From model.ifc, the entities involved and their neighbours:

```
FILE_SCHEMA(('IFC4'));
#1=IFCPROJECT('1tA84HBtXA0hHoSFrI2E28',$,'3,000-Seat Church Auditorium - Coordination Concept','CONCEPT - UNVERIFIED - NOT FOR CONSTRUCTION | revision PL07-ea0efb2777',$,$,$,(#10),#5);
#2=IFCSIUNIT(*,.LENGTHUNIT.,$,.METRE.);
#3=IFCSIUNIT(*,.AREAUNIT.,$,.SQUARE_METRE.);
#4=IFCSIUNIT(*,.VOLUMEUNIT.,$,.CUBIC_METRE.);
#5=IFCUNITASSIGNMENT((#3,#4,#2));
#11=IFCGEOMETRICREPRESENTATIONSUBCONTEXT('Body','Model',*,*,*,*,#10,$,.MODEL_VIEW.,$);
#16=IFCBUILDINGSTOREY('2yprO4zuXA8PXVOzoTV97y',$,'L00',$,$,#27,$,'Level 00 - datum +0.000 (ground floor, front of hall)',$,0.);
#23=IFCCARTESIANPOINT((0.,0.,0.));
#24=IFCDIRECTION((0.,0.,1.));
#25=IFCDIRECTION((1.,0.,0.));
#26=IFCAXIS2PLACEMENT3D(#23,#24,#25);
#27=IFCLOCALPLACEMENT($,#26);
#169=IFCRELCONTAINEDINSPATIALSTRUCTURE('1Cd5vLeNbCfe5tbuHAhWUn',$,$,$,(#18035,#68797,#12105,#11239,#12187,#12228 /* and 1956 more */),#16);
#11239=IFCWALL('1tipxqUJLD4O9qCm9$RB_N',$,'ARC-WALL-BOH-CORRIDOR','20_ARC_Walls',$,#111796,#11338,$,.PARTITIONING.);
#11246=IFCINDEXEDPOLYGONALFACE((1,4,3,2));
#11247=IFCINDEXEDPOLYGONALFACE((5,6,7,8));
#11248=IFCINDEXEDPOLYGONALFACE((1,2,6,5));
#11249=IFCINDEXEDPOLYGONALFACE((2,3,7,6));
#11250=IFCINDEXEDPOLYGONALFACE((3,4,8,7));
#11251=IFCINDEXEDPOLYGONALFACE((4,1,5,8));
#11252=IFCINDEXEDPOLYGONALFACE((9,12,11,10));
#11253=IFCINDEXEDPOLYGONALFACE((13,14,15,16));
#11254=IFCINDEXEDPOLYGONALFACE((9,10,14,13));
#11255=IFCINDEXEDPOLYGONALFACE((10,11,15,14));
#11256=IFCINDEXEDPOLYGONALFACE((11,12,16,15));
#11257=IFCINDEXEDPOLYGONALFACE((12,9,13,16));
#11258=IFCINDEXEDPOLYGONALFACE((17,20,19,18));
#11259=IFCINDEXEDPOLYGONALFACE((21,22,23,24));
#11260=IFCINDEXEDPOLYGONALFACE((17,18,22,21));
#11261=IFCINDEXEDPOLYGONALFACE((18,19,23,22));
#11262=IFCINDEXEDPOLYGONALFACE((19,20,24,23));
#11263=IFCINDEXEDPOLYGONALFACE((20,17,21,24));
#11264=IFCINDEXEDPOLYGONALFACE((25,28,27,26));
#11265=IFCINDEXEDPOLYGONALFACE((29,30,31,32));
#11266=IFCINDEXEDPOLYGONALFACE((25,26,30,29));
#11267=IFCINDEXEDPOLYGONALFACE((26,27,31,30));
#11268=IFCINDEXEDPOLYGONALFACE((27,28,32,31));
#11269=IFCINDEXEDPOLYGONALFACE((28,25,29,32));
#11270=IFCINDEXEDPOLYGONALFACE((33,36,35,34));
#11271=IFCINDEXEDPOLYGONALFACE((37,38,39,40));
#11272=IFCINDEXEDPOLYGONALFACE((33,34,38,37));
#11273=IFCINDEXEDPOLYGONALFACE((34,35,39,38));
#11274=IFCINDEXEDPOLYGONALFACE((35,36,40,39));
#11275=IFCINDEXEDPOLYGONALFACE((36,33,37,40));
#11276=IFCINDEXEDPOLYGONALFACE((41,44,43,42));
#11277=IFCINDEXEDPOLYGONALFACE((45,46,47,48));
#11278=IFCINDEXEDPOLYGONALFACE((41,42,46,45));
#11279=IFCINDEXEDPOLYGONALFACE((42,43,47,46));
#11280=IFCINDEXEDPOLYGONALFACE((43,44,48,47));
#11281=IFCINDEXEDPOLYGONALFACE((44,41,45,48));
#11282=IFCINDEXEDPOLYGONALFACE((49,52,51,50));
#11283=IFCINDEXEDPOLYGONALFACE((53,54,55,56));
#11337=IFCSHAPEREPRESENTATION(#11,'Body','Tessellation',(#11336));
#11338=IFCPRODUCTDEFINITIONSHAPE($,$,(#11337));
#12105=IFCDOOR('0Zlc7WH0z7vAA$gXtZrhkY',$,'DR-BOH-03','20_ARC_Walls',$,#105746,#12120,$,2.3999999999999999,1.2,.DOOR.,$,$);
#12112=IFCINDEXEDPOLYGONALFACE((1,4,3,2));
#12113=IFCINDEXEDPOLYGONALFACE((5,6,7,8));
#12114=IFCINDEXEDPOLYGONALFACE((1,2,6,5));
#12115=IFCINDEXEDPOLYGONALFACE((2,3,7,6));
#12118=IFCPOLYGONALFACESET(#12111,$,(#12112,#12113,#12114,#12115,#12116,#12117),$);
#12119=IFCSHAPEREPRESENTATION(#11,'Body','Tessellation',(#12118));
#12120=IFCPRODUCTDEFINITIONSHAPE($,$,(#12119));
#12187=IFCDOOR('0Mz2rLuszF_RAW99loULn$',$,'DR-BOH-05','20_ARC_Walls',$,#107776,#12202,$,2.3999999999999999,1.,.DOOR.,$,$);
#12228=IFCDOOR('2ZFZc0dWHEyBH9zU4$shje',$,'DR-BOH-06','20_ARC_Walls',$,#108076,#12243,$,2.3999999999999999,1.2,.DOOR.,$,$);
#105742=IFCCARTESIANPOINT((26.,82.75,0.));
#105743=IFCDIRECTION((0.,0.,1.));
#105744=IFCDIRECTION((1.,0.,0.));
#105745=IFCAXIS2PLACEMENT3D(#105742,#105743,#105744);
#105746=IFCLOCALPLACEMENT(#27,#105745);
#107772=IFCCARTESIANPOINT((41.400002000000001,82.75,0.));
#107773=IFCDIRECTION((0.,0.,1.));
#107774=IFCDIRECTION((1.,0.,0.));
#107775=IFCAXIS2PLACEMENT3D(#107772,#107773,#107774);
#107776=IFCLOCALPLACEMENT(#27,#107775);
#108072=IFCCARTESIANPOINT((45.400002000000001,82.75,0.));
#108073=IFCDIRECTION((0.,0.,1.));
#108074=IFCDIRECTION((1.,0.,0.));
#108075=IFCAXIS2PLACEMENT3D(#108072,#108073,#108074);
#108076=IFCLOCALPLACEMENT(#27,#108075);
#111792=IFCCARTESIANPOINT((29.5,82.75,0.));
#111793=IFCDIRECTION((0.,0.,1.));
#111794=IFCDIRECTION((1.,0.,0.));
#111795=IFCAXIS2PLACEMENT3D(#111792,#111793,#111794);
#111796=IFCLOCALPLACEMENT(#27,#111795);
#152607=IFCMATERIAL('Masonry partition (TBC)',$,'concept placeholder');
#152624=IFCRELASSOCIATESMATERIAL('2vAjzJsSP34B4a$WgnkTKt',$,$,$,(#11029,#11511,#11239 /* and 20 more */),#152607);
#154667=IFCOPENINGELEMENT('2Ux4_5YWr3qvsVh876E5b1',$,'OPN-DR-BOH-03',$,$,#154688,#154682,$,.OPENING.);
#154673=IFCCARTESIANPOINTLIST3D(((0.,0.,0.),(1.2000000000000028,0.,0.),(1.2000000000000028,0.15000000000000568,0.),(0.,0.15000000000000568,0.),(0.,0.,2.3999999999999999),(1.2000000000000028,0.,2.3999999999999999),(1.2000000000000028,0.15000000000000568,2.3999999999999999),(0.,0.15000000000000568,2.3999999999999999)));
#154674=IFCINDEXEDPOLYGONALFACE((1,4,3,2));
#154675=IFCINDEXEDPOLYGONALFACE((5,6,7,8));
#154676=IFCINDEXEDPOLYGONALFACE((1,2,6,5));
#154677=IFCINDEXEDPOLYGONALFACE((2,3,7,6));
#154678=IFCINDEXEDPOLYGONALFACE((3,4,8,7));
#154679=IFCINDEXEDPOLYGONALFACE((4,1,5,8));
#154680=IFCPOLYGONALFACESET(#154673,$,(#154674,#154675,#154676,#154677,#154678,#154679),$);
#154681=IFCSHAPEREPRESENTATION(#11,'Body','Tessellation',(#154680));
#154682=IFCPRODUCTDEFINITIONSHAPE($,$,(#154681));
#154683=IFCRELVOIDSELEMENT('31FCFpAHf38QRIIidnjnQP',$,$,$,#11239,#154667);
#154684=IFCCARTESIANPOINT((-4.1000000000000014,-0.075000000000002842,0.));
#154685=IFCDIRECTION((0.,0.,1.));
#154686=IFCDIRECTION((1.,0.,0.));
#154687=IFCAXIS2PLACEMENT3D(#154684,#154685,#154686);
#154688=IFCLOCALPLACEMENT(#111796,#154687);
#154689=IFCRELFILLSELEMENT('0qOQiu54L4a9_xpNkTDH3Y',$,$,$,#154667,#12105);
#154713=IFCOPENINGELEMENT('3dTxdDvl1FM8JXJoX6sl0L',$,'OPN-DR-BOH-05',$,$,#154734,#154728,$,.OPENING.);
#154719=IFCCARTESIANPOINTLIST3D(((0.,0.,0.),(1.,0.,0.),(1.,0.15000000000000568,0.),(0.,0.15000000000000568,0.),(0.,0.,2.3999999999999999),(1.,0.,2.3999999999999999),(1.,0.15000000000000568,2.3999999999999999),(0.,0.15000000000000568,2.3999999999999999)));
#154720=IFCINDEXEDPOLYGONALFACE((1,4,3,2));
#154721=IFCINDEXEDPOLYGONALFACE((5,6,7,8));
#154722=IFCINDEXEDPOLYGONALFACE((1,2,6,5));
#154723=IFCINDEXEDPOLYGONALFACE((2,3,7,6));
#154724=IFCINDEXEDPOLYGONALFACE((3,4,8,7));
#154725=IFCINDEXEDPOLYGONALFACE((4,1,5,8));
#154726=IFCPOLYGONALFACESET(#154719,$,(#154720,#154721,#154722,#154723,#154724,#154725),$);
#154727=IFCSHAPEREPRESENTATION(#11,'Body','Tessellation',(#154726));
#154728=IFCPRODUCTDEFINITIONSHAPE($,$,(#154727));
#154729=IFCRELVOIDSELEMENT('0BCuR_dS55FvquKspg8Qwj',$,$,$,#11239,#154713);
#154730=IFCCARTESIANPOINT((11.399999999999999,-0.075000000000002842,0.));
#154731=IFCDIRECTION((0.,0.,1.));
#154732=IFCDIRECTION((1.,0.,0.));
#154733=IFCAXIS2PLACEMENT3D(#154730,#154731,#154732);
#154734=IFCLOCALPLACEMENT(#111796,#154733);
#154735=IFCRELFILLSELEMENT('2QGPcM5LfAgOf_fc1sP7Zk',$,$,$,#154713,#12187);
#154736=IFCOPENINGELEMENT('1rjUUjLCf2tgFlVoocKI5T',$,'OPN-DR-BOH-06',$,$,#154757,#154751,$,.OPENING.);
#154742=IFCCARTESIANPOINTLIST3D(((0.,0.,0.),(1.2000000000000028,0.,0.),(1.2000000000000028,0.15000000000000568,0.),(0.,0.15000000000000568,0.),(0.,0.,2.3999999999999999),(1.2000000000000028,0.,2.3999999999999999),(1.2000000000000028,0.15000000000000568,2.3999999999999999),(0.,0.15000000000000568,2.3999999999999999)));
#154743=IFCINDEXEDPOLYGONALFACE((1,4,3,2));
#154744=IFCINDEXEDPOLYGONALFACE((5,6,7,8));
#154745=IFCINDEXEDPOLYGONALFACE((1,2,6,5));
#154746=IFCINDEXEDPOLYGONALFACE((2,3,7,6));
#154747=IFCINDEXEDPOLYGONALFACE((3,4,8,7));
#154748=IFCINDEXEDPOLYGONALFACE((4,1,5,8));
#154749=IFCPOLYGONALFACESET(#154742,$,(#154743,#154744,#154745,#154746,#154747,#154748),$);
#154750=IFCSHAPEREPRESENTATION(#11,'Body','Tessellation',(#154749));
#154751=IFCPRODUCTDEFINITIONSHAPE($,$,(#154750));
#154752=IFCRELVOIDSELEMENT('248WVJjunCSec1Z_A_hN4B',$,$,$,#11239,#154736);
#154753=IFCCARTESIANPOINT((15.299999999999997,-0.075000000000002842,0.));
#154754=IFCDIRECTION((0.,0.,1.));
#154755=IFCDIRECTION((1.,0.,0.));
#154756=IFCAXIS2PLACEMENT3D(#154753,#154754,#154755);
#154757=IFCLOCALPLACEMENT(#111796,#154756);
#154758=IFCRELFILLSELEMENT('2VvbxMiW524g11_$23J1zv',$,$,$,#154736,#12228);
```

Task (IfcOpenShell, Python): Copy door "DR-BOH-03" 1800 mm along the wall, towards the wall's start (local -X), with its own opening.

```python
import ifcopenshell
import ifcopenshell.api.feature
import ifcopenshell.api.geometry
import ifcopenshell.api.root
import ifcopenshell.geom
import ifcopenshell.util.element
import ifcopenshell.util.placement
import ifcopenshell.util.shape

model = ifcopenshell.open("model.ifc")
settings = ifcopenshell.geom.settings()


def volume(element):
    """Net volume in cubic metres, openings subtracted."""
    shape = ifcopenshell.geom.create_shape(settings, element)
    return ifcopenshell.util.shape.get_volume(shape.geometry)


door = model.by_guid("0Zlc7WH0z7vAA$gXtZrhkY")
opening = door.FillsVoids[0].RelatingOpeningElement
wall = opening.VoidsElements[0].RelatingBuildingElement
before = volume(wall)
shift = ifcopenshell.util.placement.get_local_placement(wall.ObjectPlacement)[:3, 0] * -1.8

# copy_class copies the void relationship, type, container and properties, but no geometry.
new_opening = ifcopenshell.api.root.copy_class(model, product=opening)
new_opening.Representation = ifcopenshell.util.element.copy_deep(
    model, opening.Representation, exclude=["IfcGeometricRepresentationContext", "IfcRepresentationMap"]
)
new_door = ifcopenshell.api.root.copy_class(model, product=door)
new_door.Representation = ifcopenshell.util.element.copy_deep(
    model, door.Representation, exclude=["IfcGeometricRepresentationContext", "IfcRepresentationMap"]
)
ifcopenshell.api.feature.add_filling(model, opening=new_opening, element=new_door)

for old, new in ((opening, new_opening), (door, new_door)):
    matrix = ifcopenshell.util.placement.get_local_placement(old.ObjectPlacement)
    matrix[:3, 3] += shift
    ifcopenshell.api.geometry.edit_object_placement(model, product=new, matrix=matrix, is_si=False)

after = volume(wall)

print(f"wall volume {before:.3f} -> {after:.3f} m3")

model.write("model_v2.ifc")
```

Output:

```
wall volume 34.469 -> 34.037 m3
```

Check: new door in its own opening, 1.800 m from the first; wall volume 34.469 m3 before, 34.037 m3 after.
